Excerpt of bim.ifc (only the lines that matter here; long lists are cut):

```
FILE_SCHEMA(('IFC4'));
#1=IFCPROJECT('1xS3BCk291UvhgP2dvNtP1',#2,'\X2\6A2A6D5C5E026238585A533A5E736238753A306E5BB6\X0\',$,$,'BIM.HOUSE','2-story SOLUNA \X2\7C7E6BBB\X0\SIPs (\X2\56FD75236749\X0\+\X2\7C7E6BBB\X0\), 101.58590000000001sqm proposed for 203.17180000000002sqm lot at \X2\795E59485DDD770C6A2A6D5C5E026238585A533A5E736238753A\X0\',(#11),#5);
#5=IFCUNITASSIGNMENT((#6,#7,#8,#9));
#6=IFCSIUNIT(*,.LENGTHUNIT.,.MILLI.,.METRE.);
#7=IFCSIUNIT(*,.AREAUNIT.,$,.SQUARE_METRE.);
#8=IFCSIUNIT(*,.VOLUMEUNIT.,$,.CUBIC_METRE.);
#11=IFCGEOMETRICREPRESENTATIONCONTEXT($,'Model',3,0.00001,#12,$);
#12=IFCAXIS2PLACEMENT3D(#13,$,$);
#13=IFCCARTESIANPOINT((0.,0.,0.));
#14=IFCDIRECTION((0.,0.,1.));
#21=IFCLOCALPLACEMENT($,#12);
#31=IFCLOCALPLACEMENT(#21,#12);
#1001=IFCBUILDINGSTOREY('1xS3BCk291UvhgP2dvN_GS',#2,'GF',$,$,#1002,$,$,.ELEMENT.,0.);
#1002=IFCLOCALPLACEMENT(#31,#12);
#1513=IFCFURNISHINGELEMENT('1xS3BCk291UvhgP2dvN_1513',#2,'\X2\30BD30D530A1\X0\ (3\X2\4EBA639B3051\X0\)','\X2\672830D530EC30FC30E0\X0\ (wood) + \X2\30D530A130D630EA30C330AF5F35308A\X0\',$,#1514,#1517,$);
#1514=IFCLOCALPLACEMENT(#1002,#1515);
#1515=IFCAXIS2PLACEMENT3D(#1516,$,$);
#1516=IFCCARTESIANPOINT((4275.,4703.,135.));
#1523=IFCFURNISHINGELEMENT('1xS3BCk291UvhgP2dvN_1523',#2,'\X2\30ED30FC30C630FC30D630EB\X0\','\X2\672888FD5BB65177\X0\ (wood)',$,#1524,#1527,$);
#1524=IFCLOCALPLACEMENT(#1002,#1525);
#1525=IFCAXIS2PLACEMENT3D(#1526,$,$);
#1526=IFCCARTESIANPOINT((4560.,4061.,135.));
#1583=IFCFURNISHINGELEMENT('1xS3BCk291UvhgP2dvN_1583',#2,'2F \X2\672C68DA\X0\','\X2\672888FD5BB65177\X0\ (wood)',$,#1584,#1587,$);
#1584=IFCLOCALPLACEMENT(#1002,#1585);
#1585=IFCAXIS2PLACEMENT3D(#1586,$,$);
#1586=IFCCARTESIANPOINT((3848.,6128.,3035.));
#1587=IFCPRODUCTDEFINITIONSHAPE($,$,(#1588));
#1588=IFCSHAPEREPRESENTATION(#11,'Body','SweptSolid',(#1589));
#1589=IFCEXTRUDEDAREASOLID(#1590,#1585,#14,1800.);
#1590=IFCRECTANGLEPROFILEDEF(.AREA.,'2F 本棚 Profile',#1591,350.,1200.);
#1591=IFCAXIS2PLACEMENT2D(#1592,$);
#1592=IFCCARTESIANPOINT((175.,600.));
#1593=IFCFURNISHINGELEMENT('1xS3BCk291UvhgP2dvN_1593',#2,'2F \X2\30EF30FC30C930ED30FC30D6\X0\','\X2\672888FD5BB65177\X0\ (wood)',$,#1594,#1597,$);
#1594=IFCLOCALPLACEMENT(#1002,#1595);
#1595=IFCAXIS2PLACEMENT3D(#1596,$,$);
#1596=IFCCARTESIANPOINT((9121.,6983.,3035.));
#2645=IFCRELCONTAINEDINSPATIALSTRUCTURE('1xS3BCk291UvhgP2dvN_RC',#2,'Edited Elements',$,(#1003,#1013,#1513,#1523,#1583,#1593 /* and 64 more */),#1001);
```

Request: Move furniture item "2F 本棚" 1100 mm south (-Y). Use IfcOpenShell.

```python
import ifcopenshell
import ifcopenshell.api.geometry
import ifcopenshell.util.placement
import ifcopenshell.util.unit

model = ifcopenshell.open("bim.ifc")
unit_scale = ifcopenshell.util.unit.calculate_unit_scale(model)

item = model.by_guid("1xS3BCk291UvhgP2dvN_1583")
matrix = ifcopenshell.util.placement.get_local_placement(item.ObjectPlacement)
matrix[1, 3] -= 1.1 / unit_scale
ifcopenshell.api.geometry.edit_object_placement(model, product=item, matrix=matrix, is_si=False)

print(ifcopenshell.util.placement.get_local_placement(item.ObjectPlacement).round(3) + 0.0)

model.write("bim-out.ifc")
```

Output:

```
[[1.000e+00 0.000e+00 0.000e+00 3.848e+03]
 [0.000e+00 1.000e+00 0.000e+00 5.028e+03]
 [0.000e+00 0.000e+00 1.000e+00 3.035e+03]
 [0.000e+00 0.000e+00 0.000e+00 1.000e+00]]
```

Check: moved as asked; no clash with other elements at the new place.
